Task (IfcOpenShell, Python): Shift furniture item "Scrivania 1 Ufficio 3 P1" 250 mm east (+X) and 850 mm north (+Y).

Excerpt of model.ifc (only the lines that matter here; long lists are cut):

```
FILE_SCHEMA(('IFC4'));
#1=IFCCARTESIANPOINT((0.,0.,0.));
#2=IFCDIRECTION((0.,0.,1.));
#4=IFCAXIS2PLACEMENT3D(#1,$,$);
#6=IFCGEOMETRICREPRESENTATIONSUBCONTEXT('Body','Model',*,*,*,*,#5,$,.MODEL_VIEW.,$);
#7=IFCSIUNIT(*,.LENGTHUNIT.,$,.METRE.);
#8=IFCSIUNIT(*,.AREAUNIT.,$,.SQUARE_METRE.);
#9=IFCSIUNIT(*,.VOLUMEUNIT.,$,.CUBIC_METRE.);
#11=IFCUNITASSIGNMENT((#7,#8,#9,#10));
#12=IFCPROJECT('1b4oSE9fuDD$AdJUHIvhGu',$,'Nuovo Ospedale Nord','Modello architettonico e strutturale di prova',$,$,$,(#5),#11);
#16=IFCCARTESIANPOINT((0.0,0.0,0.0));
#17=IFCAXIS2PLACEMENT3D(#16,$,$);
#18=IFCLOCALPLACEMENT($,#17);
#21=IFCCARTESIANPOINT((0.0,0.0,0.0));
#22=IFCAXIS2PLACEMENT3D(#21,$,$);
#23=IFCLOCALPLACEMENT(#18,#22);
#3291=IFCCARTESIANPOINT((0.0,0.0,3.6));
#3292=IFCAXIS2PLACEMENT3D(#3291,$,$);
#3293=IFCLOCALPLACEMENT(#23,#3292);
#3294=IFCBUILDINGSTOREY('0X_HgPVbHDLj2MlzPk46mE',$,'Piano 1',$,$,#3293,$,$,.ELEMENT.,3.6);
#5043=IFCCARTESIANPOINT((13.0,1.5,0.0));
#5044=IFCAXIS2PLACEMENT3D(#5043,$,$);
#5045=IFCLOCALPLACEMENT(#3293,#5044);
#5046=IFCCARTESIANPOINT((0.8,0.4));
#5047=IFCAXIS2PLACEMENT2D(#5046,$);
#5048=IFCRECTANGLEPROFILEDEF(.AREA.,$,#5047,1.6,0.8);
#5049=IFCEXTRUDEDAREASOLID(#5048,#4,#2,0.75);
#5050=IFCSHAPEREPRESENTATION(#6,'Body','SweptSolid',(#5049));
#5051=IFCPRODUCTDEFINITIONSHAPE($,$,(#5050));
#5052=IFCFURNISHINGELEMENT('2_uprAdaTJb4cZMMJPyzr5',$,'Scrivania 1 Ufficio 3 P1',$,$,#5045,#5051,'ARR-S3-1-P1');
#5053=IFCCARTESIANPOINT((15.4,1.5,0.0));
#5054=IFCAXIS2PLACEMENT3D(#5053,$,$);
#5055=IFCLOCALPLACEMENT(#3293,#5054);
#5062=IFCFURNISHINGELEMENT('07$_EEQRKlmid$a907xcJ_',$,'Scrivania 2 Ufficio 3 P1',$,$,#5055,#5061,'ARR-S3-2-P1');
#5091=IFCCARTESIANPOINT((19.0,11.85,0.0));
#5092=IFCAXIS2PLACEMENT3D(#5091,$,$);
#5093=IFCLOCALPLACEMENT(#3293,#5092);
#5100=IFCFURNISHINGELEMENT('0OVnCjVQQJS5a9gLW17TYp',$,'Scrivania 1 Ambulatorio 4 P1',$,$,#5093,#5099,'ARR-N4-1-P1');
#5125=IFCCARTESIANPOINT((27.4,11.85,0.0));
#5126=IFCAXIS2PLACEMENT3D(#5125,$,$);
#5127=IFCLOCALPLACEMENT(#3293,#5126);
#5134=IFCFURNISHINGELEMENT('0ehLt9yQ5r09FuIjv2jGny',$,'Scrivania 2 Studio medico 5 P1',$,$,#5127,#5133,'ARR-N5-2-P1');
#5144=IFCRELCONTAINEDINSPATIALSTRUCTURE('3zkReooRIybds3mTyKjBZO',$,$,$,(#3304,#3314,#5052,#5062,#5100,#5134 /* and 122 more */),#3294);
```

```python
import ifcopenshell
import ifcopenshell.api.geometry
import ifcopenshell.util.placement

model = ifcopenshell.open("model.ifc")

item = model.by_guid("2_uprAdaTJb4cZMMJPyzr5")
matrix = ifcopenshell.util.placement.get_local_placement(item.ObjectPlacement)
matrix[0, 3] += 0.25
matrix[1, 3] += 0.85
ifcopenshell.api.geometry.edit_object_placement(model, product=item, matrix=matrix, is_si=False)

print(ifcopenshell.util.placement.get_local_placement(item.ObjectPlacement).round(3) + 0.0)

model.write("model_v2.ifc")
```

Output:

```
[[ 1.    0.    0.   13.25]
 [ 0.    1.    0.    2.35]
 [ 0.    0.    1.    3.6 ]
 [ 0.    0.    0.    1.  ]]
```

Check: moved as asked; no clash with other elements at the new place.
